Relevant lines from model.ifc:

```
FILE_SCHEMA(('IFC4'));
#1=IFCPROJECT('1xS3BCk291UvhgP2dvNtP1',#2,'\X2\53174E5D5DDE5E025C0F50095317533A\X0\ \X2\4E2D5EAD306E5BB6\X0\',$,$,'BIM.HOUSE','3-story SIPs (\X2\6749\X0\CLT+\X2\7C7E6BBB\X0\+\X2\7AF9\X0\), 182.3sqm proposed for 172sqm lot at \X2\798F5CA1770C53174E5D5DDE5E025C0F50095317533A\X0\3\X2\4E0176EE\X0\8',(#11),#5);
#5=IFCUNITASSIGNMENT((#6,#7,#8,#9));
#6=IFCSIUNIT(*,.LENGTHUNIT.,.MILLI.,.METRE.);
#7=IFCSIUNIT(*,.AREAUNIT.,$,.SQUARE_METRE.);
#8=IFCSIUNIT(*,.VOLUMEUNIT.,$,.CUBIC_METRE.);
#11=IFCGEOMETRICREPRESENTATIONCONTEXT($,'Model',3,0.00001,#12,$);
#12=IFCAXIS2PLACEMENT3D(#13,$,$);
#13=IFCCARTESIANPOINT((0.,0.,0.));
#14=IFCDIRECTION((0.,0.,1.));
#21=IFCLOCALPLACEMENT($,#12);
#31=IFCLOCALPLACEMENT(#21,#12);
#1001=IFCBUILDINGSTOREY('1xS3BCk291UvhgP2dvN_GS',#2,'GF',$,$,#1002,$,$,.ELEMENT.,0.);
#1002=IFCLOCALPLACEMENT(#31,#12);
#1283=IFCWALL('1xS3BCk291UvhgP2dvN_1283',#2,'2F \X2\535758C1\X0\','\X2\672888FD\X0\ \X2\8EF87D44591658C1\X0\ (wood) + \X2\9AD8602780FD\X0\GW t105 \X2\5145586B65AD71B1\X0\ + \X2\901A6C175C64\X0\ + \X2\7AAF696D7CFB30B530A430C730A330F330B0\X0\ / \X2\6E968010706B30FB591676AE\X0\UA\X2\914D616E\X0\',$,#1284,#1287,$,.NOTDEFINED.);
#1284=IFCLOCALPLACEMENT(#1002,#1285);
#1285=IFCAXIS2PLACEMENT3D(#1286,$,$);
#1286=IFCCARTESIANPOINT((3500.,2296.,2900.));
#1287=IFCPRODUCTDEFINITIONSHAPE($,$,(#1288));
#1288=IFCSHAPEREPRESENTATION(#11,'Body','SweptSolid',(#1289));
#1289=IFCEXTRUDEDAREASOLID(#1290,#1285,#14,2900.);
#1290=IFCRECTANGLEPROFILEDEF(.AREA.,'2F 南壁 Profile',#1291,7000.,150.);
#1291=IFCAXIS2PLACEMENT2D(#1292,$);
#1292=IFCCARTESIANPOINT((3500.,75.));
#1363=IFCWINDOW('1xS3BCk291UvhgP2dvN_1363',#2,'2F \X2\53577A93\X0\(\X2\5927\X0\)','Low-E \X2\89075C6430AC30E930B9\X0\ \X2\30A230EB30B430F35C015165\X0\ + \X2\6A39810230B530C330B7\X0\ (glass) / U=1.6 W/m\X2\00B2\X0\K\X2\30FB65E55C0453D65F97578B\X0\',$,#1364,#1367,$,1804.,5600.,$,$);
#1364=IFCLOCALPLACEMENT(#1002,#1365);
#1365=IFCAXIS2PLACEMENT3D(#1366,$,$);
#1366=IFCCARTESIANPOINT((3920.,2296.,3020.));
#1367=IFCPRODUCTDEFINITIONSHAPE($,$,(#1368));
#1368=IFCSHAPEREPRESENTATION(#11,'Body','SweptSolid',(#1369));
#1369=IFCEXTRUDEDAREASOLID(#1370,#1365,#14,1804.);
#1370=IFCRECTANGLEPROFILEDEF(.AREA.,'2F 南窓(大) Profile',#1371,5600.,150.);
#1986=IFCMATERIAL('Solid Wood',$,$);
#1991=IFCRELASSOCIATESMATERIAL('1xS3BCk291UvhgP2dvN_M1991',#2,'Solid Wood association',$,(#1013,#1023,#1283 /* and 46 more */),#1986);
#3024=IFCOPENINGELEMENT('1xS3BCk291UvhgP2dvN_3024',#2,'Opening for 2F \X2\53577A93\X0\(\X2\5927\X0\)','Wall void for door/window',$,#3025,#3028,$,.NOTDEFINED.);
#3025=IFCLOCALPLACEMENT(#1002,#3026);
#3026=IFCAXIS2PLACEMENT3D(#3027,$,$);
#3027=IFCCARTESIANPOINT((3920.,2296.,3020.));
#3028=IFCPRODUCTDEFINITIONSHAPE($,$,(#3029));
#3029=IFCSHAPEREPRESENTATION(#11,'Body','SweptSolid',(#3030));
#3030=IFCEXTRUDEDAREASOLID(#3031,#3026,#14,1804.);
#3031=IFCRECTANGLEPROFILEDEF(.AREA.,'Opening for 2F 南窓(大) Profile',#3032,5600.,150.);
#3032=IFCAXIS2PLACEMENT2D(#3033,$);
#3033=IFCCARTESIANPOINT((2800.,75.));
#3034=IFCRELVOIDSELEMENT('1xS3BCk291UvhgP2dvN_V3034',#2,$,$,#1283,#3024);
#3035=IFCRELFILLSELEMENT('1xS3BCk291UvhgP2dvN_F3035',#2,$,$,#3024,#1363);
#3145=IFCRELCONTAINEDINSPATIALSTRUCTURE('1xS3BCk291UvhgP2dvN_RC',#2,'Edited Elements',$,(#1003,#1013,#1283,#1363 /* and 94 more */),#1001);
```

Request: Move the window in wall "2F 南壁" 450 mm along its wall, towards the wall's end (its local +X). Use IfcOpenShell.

```python
import ifcopenshell
import ifcopenshell.api.geometry
import ifcopenshell.util.placement
import ifcopenshell.util.unit

model = ifcopenshell.open("model.ifc")
unit_scale = ifcopenshell.util.unit.calculate_unit_scale(model)

window = model.by_guid("1xS3BCk291UvhgP2dvN_1363")
opening = window.FillsVoids[0].RelatingOpeningElement
wall = opening.VoidsElements[0].RelatingBuildingElement

wall_matrix = ifcopenshell.util.placement.get_local_placement(wall.ObjectPlacement)
shift = wall_matrix[:3, 0] * 0.45 / unit_scale
before = ifcopenshell.util.placement.get_local_placement(window.ObjectPlacement)[:3, 3].copy()

# The window is not placed relative to its opening, so move both.
for product in (opening, window):
    matrix = ifcopenshell.util.placement.get_local_placement(product.ObjectPlacement)
    matrix[:3, 3] += shift
    ifcopenshell.api.geometry.edit_object_placement(model, product=product, matrix=matrix, is_si=False)

after = ifcopenshell.util.placement.get_local_placement(window.ObjectPlacement)[:3, 3]
print("window moved by", (after - before).round(3) + 0.0)

model.write("model_edited.ifc")
```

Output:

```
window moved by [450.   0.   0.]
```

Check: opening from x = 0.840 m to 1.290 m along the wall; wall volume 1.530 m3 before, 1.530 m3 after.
